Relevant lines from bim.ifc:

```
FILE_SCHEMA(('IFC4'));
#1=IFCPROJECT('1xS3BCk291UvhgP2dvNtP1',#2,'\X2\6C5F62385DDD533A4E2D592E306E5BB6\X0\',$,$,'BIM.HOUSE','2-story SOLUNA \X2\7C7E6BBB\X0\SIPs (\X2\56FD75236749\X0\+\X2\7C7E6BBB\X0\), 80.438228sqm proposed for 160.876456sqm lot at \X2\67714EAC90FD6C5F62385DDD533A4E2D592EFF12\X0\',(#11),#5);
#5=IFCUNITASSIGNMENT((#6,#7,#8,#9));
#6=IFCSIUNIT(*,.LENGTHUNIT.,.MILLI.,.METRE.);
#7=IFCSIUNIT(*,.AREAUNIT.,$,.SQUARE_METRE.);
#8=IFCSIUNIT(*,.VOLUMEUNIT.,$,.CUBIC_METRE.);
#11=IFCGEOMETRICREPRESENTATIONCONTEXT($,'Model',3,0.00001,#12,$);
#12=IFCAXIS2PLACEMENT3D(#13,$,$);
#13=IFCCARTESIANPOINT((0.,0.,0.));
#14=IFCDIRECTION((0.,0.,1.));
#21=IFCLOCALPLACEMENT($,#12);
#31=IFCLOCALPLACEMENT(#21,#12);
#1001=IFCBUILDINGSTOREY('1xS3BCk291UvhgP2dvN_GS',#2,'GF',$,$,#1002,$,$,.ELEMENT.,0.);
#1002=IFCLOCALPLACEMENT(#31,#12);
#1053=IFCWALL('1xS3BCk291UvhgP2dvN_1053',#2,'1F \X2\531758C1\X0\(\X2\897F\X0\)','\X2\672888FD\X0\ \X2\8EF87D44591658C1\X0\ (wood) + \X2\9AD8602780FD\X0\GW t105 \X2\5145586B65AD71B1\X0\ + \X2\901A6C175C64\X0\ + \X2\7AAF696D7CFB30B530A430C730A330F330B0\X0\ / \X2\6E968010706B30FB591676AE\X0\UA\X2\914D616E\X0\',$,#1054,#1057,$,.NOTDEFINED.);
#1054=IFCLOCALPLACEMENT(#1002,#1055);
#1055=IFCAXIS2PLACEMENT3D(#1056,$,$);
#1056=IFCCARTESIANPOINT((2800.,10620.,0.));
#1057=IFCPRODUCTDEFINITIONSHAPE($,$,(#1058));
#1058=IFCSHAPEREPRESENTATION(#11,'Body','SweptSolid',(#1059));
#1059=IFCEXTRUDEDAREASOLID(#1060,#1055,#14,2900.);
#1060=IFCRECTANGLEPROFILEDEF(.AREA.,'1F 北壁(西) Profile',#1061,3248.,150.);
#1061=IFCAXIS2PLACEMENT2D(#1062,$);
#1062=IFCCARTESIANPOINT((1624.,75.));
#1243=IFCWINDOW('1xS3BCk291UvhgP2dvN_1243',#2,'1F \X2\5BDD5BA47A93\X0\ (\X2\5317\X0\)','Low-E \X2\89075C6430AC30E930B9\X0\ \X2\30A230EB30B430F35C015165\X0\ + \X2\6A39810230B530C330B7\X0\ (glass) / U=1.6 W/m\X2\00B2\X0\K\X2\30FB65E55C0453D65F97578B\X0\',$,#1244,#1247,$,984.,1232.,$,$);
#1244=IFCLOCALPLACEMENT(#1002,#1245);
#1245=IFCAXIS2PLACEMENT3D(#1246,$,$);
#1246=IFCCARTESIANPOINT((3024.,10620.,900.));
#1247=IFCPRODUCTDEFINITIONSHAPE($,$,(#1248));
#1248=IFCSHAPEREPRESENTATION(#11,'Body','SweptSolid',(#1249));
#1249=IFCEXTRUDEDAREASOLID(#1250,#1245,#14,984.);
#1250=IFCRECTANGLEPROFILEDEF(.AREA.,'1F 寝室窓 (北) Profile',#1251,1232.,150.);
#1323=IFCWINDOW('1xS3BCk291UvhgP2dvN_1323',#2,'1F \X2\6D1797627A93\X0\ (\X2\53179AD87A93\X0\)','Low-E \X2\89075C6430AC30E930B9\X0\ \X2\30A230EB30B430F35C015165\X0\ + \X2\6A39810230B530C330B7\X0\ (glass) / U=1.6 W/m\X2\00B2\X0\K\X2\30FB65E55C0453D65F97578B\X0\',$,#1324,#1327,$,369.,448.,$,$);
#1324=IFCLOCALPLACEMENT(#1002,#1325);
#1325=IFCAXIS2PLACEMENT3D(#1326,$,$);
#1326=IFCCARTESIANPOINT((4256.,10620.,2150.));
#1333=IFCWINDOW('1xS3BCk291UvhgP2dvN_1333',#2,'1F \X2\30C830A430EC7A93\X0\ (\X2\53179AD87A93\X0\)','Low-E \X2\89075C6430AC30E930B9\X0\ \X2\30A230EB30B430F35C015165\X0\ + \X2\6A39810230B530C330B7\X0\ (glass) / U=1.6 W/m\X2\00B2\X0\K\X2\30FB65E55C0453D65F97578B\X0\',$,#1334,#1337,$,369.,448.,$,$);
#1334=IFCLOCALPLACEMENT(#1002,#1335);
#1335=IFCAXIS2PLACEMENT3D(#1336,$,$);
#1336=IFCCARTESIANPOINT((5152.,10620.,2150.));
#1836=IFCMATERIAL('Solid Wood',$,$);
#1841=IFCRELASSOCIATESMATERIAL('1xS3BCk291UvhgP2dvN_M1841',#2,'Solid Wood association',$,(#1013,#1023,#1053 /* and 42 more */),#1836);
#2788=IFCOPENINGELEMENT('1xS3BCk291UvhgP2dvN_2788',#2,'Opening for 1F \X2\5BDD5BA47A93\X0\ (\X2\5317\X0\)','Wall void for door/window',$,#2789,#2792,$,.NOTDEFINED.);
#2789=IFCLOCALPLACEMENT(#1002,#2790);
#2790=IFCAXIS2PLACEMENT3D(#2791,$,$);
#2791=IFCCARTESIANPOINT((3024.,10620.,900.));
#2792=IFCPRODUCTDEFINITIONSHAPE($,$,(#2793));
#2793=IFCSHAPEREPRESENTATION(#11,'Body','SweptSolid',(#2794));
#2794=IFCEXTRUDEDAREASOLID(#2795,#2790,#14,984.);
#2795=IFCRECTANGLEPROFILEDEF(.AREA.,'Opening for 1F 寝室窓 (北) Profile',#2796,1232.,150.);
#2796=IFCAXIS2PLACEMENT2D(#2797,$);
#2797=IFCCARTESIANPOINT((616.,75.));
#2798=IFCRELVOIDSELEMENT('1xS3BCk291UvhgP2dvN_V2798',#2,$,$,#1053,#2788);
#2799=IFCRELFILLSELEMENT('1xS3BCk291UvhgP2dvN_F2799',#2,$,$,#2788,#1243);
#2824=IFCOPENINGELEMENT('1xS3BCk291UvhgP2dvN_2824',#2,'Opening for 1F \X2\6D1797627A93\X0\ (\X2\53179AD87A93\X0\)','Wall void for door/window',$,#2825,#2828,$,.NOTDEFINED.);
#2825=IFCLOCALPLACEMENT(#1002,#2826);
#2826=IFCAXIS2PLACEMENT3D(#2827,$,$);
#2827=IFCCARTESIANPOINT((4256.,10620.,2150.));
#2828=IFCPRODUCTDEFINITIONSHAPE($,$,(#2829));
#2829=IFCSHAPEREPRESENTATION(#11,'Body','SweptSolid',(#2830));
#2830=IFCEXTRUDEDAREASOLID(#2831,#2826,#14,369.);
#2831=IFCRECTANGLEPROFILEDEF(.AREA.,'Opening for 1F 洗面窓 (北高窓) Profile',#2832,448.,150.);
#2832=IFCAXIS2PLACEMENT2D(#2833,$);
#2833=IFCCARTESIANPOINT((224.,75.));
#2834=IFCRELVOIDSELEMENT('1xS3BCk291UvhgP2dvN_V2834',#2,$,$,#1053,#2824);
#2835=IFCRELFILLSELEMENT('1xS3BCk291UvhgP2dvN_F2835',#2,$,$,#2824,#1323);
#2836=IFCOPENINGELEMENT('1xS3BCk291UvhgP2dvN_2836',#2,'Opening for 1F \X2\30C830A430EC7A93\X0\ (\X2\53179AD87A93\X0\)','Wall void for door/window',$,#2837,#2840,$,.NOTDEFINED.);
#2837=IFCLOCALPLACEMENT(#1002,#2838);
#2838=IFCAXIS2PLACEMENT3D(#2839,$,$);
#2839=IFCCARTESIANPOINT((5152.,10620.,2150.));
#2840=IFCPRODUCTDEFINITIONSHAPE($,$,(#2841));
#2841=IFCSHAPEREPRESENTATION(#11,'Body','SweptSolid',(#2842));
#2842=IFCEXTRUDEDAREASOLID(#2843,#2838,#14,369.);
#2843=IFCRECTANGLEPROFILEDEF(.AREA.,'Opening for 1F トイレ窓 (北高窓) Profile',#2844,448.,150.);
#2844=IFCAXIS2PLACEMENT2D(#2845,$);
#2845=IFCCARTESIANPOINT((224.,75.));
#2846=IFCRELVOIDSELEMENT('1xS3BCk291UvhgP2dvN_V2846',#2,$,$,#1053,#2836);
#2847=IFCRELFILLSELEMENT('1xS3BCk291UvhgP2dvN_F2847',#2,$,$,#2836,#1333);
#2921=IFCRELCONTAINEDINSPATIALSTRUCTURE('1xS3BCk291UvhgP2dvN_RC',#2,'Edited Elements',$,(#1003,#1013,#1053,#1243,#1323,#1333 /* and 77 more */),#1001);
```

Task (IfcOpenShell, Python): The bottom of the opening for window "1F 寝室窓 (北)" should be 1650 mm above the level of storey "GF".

```python
import numpy as np
import ifcopenshell
import ifcopenshell.api.geometry
import ifcopenshell.geom
import ifcopenshell.util.element
import ifcopenshell.util.placement
import ifcopenshell.util.shape
import ifcopenshell.util.unit

model = ifcopenshell.open("bim.ifc")
unit_scale = ifcopenshell.util.unit.calculate_unit_scale(model)

window = model.by_guid("1xS3BCk291UvhgP2dvN_1243")
opening = window.FillsVoids[0].RelatingOpeningElement
storey = ifcopenshell.util.element.get_container(window, ifc_class="IfcBuildingStorey")
level = ifcopenshell.util.placement.get_local_placement(storey.ObjectPlacement)[2, 3]

# The opening's origin need not be at the sill, so measure its lowest point.
shape = ifcopenshell.geom.create_shape(ifcopenshell.geom.settings(), opening)
bottom = ifcopenshell.util.shape.get_shape_bottom_elevation(shape, shape.geometry) / unit_scale
dz = level + 1650.0 - bottom

shift = np.array([0.0, 0.0, dz])
# The window is not placed relative to its opening, so move both.
for product in (opening, window):
    matrix = ifcopenshell.util.placement.get_local_placement(product.ObjectPlacement)
    matrix[:3, 3] += shift
    ifcopenshell.api.geometry.edit_object_placement(model, product=product, matrix=matrix, is_si=False)

print(f"moved by {dz * unit_scale:+.3f} m")

model.write("bim_edited.ifc")
```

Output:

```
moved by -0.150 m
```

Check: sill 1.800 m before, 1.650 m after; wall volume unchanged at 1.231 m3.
